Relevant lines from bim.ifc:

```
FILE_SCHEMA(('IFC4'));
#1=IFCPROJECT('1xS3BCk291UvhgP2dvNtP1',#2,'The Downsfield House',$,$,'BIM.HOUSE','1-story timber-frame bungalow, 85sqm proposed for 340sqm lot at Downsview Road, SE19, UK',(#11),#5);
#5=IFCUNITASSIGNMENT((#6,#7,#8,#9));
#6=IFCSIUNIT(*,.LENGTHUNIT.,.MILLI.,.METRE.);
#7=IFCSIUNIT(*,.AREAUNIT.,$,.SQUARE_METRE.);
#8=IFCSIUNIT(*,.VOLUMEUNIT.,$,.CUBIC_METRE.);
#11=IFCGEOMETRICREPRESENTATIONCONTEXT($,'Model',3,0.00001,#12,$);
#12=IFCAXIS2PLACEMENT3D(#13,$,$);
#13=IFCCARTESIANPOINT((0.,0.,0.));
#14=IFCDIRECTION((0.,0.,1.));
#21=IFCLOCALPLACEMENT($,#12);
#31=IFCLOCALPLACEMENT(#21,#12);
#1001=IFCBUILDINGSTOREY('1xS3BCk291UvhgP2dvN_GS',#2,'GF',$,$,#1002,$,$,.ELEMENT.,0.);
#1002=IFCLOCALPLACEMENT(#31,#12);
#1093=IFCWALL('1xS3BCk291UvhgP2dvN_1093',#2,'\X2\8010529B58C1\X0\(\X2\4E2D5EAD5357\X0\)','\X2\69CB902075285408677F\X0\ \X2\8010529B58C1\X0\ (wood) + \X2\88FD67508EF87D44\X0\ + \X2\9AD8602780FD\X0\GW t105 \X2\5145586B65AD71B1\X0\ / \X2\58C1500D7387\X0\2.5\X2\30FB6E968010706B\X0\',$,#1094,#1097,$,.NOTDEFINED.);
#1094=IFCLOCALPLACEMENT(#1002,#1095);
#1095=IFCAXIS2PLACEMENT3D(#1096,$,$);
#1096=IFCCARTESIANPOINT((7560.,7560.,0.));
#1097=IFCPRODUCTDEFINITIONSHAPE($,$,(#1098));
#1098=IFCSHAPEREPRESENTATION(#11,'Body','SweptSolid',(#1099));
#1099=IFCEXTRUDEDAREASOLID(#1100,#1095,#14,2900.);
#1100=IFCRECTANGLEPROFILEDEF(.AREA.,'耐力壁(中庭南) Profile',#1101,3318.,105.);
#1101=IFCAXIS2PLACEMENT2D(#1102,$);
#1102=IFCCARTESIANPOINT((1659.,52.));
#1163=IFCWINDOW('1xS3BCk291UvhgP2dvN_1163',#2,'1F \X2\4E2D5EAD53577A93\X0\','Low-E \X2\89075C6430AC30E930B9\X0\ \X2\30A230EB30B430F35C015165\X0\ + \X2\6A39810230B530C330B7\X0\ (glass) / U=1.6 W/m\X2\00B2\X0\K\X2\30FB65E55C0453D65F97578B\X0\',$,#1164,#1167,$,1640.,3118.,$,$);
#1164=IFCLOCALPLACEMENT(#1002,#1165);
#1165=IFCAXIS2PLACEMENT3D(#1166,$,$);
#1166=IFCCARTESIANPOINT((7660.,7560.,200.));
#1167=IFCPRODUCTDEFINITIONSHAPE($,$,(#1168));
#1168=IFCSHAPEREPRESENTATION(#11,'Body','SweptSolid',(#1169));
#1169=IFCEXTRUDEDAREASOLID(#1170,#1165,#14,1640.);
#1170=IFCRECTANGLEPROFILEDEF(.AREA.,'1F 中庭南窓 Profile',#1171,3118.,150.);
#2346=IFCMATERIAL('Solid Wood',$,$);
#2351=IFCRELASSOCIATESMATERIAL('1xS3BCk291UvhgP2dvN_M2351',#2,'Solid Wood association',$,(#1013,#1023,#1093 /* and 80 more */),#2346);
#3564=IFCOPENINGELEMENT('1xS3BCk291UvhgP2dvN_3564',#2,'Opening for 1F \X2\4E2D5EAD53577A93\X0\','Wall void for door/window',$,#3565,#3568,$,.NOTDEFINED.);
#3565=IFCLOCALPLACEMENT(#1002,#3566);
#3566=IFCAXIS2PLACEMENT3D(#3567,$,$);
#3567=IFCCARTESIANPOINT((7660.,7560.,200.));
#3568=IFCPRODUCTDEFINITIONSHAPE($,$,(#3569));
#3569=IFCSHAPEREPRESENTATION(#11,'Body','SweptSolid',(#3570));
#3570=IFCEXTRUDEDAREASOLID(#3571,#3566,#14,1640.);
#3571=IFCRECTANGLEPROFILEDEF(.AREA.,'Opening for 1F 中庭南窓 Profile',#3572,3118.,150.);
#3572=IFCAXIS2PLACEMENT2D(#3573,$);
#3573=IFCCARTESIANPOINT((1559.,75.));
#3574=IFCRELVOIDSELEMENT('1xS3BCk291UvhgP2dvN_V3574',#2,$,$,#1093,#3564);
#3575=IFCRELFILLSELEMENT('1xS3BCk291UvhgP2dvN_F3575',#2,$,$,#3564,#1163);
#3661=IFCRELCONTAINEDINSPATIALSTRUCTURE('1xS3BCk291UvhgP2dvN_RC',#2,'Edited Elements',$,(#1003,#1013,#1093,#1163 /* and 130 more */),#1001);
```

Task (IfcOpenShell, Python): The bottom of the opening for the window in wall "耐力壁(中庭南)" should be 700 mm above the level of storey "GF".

```python
import numpy as np
import ifcopenshell
import ifcopenshell.api.geometry
import ifcopenshell.geom
import ifcopenshell.util.element
import ifcopenshell.util.placement
import ifcopenshell.util.shape
import ifcopenshell.util.unit

model = ifcopenshell.open("bim.ifc")
unit_scale = ifcopenshell.util.unit.calculate_unit_scale(model)

window = model.by_guid("1xS3BCk291UvhgP2dvN_1163")
opening = window.FillsVoids[0].RelatingOpeningElement
storey = ifcopenshell.util.element.get_container(window, ifc_class="IfcBuildingStorey")
level = ifcopenshell.util.placement.get_local_placement(storey.ObjectPlacement)[2, 3]

# The opening's origin need not be at the sill, so measure its lowest point.
shape = ifcopenshell.geom.create_shape(ifcopenshell.geom.settings(), opening)
bottom = ifcopenshell.util.shape.get_shape_bottom_elevation(shape, shape.geometry) / unit_scale
dz = level + 0.7 / unit_scale - bottom

shift = np.array([0.0, 0.0, dz])
# The window is not placed relative to its opening, so move both.
for product in (opening, window):
    matrix = ifcopenshell.util.placement.get_local_placement(product.ObjectPlacement)
    matrix[:3, 3] += shift
    ifcopenshell.api.geometry.edit_object_placement(model, product=product, matrix=matrix, is_si=False)

print(f"moved by {dz * unit_scale:+.3f} m")

model.write("bim_edited.ifc")
```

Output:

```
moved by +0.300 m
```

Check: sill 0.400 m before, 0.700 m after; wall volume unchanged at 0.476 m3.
